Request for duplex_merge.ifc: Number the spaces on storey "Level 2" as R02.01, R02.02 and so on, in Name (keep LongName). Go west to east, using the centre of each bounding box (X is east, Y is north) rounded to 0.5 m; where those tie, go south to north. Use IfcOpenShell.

First a look at what the model holds.

```python
import ifcopenshell
import ifcopenshell.util.element
import ifcopenshell.util.placement

model = ifcopenshell.open("duplex_merge.ifc")
print(model.schema)
storey = next(s for s in model.by_type("IfcBuildingStorey") if s.Name == "Level 2")
spaces = [e for e in ifcopenshell.util.element.get_decomposition(storey) if e.is_a("IfcSpace")]
for e in sorted(spaces, key=lambda e: e.id()):
    origin = ifcopenshell.util.placement.get_local_placement(e.ObjectPlacement)[:3, 3]
    print(e.id(), e.Name, e.LongName, origin.round(2) + 0.0, sep=" | ")
```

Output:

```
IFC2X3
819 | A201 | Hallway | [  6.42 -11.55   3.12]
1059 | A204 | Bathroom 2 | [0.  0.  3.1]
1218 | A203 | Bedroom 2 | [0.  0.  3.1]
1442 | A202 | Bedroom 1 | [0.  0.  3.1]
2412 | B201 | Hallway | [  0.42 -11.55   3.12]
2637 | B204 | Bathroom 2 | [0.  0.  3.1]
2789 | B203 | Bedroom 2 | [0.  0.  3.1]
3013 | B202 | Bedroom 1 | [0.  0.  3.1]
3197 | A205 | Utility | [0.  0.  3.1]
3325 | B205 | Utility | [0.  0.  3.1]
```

```python
import ifcopenshell
import ifcopenshell.geom
import ifcopenshell.util.element
import ifcopenshell.util.shape

model = ifcopenshell.open("duplex_merge.ifc")
settings = ifcopenshell.geom.settings()
settings.set("use-world-coords", True)


def centre(element):
    shape = ifcopenshell.geom.create_shape(settings, element)
    return ifcopenshell.util.shape.get_bbox_centroid(shape.geometry)


storey = next(s for s in model.by_type("IfcBuildingStorey") if s.Name == "Level 2")
spaces = [e for e in ifcopenshell.util.element.get_decomposition(storey) if e.is_a("IfcSpace")]

# Insertion points can sit at a corner or the storey origin, so sort by the geometry (in metres).
centres = {e: centre(e) for e in spaces}
spaces.sort(key=lambda e: (round(centres[e][0] / 0.5), centres[e][1]))

for i, e in enumerate(spaces, start=1):
    number = f"R02.{i:02d}"
    e.Name = number
    print(e.id(), number)

model.write("duplex_merge_updated.ifc")
```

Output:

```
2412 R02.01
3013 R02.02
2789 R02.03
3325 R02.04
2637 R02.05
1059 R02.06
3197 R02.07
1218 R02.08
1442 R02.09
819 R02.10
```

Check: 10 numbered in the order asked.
